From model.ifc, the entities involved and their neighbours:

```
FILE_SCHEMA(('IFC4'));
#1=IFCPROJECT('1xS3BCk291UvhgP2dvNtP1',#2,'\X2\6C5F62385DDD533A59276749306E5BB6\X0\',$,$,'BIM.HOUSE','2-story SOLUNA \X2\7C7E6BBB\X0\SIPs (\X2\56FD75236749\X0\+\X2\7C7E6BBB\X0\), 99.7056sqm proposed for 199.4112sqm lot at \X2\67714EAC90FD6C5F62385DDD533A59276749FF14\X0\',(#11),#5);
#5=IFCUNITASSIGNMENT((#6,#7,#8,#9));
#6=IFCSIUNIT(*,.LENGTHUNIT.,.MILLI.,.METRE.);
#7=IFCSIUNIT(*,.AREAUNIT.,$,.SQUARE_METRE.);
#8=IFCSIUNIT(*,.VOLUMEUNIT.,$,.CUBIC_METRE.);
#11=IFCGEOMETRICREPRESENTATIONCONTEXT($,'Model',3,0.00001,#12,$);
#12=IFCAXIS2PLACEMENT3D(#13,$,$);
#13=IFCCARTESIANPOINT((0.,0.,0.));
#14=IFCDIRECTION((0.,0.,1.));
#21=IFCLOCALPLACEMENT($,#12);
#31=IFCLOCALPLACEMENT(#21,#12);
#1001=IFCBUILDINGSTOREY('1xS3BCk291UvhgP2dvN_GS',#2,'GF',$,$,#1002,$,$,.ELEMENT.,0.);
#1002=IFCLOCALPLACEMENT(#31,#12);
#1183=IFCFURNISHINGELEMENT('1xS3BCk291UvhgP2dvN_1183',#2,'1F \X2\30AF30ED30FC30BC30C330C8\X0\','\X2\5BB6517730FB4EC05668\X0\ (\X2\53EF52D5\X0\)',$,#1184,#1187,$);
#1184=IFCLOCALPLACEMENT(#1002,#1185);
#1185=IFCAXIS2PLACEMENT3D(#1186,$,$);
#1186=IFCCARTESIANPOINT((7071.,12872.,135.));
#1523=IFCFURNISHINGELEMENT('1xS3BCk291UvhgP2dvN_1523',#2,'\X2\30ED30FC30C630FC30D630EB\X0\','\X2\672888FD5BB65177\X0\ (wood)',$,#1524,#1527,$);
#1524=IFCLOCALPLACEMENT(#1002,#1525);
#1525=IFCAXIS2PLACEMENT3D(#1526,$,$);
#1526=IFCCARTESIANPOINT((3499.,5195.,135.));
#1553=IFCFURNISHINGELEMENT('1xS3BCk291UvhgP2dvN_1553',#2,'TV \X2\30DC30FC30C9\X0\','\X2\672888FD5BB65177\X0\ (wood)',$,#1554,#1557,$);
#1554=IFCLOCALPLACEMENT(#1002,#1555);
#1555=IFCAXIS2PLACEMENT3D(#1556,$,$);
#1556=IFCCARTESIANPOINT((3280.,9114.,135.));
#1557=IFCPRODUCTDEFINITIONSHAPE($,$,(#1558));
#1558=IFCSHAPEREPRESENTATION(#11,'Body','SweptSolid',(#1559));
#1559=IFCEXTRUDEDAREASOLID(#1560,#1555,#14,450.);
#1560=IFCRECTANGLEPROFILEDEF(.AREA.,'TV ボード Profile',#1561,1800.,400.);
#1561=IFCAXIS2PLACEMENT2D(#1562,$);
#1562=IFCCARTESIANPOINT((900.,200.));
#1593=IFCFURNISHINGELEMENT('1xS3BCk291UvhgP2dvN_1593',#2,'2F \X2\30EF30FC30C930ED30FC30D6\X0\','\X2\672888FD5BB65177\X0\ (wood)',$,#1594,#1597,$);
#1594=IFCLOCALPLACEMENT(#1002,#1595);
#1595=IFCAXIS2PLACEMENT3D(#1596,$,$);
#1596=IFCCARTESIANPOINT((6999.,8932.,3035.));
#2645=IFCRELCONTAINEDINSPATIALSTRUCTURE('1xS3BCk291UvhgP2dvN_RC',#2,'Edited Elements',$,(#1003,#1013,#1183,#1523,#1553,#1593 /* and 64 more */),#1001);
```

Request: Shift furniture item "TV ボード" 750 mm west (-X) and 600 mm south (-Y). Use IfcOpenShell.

```python
import ifcopenshell
import ifcopenshell.api.geometry
import ifcopenshell.util.placement
import ifcopenshell.util.unit

model = ifcopenshell.open("model.ifc")
unit_scale = ifcopenshell.util.unit.calculate_unit_scale(model)

item = model.by_guid("1xS3BCk291UvhgP2dvN_1553")
matrix = ifcopenshell.util.placement.get_local_placement(item.ObjectPlacement)
matrix[0, 3] -= 0.75 / unit_scale
matrix[1, 3] -= 0.6 / unit_scale
ifcopenshell.api.geometry.edit_object_placement(model, product=item, matrix=matrix, is_si=False)

print(ifcopenshell.util.placement.get_local_placement(item.ObjectPlacement).round(3) + 0.0)

model.write("model_v2.ifc")
```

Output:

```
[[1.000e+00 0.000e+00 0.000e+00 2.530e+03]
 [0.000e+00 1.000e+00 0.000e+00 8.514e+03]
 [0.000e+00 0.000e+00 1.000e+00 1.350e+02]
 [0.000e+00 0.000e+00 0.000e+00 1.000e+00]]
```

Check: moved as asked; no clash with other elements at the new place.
